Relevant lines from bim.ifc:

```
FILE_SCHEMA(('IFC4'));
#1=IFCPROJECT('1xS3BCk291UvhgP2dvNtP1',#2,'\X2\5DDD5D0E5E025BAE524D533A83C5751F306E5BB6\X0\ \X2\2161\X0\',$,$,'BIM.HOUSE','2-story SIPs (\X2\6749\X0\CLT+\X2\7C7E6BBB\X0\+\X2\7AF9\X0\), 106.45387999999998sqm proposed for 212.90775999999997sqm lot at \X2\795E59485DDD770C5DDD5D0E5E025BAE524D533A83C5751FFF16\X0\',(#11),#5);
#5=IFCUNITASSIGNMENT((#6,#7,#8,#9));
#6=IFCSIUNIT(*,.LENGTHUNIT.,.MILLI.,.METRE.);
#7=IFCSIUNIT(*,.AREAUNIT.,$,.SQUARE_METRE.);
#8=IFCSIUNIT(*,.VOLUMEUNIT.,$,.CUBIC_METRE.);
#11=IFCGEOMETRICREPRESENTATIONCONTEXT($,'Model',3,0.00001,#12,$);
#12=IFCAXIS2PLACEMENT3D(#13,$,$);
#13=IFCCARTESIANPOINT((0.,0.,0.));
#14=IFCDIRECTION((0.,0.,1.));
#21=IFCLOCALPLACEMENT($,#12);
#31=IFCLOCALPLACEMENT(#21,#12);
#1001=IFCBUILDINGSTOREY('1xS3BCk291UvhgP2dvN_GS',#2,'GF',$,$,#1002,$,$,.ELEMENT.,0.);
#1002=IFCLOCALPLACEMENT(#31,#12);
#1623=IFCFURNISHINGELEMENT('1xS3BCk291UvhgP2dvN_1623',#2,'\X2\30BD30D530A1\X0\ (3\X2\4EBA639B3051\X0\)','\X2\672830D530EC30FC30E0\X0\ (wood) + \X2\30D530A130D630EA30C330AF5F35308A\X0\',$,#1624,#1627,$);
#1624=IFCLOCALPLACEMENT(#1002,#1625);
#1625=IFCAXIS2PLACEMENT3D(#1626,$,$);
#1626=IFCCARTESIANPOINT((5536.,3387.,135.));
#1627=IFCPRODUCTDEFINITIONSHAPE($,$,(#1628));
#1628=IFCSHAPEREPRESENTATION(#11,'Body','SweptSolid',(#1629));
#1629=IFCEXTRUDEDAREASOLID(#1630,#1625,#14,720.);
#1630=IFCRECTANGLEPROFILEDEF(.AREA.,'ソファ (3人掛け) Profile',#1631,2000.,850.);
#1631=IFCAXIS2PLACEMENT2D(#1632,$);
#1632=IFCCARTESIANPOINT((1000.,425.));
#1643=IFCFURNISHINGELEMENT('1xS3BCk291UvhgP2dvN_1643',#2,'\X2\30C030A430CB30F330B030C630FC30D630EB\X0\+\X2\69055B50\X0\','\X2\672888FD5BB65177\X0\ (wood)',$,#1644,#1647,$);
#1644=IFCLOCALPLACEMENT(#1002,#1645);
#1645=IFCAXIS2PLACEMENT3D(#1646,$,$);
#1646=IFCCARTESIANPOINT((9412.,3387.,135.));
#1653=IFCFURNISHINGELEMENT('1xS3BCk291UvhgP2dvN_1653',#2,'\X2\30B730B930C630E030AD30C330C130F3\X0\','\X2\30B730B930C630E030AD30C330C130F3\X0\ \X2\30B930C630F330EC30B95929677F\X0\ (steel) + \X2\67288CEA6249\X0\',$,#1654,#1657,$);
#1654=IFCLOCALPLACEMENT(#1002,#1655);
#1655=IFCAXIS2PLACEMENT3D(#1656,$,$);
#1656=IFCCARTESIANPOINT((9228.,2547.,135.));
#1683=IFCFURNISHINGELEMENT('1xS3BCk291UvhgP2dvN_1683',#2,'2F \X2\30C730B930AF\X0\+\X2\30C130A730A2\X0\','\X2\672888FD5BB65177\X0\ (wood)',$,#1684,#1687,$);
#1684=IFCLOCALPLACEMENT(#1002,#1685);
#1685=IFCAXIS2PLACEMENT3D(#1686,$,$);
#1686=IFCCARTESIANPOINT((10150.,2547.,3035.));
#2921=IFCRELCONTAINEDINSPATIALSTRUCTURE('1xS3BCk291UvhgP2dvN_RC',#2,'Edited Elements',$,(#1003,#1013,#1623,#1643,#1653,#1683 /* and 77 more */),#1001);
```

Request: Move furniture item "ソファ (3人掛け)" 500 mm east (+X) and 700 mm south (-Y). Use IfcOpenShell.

```python
import ifcopenshell
import ifcopenshell.api.geometry
import ifcopenshell.util.placement

model = ifcopenshell.open("bim.ifc")

item = model.by_guid("1xS3BCk291UvhgP2dvN_1623")
matrix = ifcopenshell.util.placement.get_local_placement(item.ObjectPlacement)
matrix[0, 3] += 500.0
matrix[1, 3] -= 700.0
ifcopenshell.api.geometry.edit_object_placement(model, product=item, matrix=matrix, is_si=False)

print(ifcopenshell.util.placement.get_local_placement(item.ObjectPlacement).round(3) + 0.0)

model.write("bim-out.ifc")
```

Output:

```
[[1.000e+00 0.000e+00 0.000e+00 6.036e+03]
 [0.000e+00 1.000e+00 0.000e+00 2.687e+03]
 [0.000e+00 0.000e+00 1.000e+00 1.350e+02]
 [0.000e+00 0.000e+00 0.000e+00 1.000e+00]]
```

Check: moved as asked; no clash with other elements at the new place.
